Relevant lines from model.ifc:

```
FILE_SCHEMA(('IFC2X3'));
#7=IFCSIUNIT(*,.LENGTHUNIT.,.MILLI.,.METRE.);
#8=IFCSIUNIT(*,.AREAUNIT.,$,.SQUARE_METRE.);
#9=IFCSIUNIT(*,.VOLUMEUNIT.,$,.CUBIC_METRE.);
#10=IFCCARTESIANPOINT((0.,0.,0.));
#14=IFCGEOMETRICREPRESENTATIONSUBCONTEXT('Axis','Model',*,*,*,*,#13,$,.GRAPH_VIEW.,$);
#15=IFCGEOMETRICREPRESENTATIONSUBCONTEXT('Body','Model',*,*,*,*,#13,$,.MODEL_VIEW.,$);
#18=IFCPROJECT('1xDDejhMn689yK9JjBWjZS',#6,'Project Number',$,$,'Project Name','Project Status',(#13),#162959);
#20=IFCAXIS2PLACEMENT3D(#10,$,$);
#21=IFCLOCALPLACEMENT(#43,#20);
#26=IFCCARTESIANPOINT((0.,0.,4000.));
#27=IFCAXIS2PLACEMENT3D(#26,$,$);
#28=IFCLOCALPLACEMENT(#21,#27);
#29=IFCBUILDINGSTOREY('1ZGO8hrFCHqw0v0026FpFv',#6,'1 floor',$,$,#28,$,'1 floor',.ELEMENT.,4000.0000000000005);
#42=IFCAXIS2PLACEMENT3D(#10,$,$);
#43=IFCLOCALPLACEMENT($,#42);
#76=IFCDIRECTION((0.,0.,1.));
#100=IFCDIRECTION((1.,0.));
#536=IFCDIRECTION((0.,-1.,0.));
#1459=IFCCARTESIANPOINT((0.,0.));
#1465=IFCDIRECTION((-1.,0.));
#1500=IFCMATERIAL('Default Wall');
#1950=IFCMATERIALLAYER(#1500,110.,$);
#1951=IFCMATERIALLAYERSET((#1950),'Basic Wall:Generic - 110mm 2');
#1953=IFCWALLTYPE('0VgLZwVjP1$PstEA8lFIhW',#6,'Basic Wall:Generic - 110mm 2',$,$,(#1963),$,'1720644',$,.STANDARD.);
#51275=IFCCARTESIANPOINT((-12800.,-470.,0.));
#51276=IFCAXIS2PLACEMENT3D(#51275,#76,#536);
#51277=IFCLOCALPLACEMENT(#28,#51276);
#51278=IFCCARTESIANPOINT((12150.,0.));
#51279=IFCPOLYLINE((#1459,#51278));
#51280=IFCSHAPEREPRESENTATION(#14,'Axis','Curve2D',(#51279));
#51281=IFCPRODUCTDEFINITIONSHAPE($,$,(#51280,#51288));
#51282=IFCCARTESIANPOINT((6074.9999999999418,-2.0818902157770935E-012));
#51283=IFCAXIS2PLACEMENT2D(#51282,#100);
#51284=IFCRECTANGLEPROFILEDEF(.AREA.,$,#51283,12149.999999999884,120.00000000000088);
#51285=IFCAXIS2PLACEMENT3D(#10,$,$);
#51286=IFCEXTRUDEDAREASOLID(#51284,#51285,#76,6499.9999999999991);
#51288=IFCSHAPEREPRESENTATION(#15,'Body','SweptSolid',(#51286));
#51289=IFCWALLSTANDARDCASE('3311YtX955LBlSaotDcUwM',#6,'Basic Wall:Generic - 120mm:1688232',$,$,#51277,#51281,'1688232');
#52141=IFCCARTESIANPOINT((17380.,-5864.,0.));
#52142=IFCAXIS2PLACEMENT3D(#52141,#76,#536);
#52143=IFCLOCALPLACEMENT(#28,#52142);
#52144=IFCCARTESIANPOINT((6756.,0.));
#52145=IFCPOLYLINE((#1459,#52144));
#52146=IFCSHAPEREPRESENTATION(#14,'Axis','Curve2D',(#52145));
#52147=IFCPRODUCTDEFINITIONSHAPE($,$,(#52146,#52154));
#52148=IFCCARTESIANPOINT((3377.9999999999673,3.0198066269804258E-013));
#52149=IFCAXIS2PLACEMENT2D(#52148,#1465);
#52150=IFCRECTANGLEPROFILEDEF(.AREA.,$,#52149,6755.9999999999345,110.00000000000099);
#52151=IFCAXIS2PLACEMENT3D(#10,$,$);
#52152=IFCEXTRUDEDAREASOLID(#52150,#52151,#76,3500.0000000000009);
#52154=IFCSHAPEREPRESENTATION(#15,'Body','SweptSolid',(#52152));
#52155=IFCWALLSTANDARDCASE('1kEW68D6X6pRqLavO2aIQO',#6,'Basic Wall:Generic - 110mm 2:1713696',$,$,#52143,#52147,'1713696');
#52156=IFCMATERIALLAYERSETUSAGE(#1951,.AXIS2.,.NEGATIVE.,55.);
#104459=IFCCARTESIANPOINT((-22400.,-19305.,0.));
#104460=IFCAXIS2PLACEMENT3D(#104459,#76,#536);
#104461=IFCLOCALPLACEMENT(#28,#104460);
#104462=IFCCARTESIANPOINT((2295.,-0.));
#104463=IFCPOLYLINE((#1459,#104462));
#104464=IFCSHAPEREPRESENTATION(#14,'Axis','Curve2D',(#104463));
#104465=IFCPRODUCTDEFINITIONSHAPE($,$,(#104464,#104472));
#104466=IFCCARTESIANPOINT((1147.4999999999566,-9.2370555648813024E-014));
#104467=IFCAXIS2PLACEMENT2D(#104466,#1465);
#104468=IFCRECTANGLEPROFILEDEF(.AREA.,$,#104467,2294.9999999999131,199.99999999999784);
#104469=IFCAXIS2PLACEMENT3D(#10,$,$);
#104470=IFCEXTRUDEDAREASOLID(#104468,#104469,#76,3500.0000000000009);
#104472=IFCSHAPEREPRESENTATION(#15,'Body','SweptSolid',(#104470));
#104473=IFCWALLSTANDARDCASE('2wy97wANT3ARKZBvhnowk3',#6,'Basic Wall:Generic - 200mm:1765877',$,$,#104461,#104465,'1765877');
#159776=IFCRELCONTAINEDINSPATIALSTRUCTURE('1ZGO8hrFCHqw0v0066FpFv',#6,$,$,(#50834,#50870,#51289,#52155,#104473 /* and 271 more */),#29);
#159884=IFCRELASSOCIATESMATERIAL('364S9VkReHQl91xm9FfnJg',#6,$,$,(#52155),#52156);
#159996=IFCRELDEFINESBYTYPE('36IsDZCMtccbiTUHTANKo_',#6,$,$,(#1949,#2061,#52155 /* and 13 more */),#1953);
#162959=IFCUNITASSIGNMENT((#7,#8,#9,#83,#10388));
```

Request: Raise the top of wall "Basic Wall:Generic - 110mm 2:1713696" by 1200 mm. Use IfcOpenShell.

```python
import ifcopenshell
import ifcopenshell.geom
import ifcopenshell.util.representation
import ifcopenshell.util.shape
import ifcopenshell.util.unit

model = ifcopenshell.open("model.ifc")
unit_scale = ifcopenshell.util.unit.calculate_unit_scale(model)
settings = ifcopenshell.geom.settings()


def volume(element):
    """Net volume in cubic metres, openings subtracted."""
    shape = ifcopenshell.geom.create_shape(settings, element)
    return ifcopenshell.util.shape.get_volume(shape.geometry)


wall = model.by_guid("1kEW68D6X6pRqLavO2aIQO")
before = volume(wall)

body = ifcopenshell.util.representation.get_representation(wall, "Model", "Body")
solid = body.Items[0]
old_height = solid.Depth
solid.Depth += 1.2 / unit_scale
after = volume(wall)

print(f"height {old_height:g} -> {solid.Depth:g}, volume {before:.3f} -> {after:.3f} m3")

model.write("model_updated.ifc")
```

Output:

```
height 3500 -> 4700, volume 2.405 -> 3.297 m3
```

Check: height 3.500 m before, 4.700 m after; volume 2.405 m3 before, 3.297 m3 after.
